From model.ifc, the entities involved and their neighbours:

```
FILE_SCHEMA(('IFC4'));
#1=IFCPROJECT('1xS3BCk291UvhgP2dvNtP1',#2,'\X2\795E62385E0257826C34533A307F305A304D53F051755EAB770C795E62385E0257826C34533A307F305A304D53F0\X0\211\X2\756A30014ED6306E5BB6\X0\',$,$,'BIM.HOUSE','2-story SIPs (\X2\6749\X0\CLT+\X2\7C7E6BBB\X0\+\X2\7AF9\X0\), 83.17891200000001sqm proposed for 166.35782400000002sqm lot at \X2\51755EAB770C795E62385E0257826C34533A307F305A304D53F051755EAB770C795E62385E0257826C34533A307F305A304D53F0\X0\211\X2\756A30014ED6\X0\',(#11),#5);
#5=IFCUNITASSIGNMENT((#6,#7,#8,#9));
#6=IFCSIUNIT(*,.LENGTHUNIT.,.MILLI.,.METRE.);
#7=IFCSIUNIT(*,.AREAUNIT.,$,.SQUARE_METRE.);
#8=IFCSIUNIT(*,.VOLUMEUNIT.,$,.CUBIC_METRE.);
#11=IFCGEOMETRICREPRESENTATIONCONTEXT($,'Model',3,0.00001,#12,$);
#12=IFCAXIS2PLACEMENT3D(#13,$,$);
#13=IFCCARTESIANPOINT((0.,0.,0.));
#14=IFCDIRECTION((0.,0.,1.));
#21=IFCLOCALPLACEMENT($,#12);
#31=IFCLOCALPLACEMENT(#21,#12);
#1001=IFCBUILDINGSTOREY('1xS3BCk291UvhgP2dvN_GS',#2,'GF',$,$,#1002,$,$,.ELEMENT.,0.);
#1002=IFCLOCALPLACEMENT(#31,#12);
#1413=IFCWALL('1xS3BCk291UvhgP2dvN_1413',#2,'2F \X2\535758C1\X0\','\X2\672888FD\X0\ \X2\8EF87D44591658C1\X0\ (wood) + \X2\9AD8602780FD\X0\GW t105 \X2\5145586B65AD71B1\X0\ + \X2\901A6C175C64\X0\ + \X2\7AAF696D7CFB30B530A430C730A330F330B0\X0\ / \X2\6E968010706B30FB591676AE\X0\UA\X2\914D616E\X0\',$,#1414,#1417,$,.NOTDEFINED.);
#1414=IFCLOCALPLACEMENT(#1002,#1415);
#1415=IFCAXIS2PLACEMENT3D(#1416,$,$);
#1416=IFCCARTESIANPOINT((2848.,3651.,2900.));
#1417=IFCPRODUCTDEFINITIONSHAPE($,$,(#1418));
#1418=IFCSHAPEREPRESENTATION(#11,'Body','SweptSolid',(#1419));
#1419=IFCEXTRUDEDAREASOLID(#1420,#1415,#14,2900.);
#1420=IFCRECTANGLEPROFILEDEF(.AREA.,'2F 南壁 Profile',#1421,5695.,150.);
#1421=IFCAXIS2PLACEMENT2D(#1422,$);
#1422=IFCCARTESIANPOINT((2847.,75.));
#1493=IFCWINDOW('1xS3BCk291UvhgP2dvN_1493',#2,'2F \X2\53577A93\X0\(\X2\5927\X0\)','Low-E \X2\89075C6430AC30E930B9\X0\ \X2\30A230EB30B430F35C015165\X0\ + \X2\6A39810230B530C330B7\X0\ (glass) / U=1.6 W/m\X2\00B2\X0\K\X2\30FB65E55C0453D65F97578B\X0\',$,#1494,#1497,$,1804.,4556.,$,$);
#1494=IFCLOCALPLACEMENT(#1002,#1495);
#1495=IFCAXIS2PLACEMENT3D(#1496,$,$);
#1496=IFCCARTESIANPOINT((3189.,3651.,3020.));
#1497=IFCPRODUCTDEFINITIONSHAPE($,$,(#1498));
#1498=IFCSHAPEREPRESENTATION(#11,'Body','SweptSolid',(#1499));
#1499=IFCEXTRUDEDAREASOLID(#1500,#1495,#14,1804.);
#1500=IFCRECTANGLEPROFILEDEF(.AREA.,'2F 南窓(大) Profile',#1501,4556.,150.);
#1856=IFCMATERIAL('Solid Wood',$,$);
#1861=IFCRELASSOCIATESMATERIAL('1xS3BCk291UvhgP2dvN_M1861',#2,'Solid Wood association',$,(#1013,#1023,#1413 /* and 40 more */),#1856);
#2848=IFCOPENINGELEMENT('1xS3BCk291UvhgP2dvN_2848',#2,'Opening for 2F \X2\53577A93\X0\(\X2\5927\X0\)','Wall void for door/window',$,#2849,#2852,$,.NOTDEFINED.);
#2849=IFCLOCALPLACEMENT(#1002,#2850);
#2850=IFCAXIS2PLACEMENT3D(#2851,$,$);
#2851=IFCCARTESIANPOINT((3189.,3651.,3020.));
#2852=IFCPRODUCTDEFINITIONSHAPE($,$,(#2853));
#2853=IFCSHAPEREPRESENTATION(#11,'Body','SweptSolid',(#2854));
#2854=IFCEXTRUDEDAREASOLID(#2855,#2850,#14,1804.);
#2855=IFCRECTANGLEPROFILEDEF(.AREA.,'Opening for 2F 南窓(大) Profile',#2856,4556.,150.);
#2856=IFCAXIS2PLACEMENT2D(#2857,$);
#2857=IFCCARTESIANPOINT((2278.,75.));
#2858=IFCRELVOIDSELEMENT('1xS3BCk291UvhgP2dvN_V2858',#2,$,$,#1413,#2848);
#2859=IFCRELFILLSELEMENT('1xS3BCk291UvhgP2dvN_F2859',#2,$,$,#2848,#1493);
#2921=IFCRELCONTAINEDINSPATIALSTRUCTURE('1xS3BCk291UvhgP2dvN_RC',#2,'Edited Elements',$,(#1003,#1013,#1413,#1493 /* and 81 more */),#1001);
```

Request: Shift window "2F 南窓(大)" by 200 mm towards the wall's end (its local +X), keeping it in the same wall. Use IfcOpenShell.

```python
import ifcopenshell
import ifcopenshell.api.geometry
import ifcopenshell.util.placement
import ifcopenshell.util.unit

model = ifcopenshell.open("model.ifc")
unit_scale = ifcopenshell.util.unit.calculate_unit_scale(model)

window = model.by_guid("1xS3BCk291UvhgP2dvN_1493")
opening = window.FillsVoids[0].RelatingOpeningElement
wall = opening.VoidsElements[0].RelatingBuildingElement

wall_matrix = ifcopenshell.util.placement.get_local_placement(wall.ObjectPlacement)
shift = wall_matrix[:3, 0] * 0.2 / unit_scale
before = ifcopenshell.util.placement.get_local_placement(window.ObjectPlacement)[:3, 3].copy()

# The window is not placed relative to its opening, so move both.
for product in (opening, window):
    matrix = ifcopenshell.util.placement.get_local_placement(product.ObjectPlacement)
    matrix[:3, 3] += shift
    ifcopenshell.api.geometry.edit_object_placement(model, product=product, matrix=matrix, is_si=False)

after = ifcopenshell.util.placement.get_local_placement(window.ObjectPlacement)[:3, 3]
print("window moved by", (after - before).round(3) + 0.0)

model.write("model_rev.ifc")
```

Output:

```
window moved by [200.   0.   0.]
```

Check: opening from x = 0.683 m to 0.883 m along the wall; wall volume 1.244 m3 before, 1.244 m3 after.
